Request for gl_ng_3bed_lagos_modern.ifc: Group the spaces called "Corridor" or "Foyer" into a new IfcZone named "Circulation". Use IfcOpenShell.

First a look at what the model holds.

```python
import ifcopenshell

model = ifcopenshell.open("gl_ng_3bed_lagos_modern.ifc")
print(model.schema)
seen = {}
for space in model.by_type("IfcSpace"):
    seen[space.LongName] = seen.get(space.LongName, 0) + 1
for name, count in sorted(seen.items(), key=str):
    print(count, "x", name)
print("zones:", [z.Name for z in model.by_type("IfcZone")][:20])
```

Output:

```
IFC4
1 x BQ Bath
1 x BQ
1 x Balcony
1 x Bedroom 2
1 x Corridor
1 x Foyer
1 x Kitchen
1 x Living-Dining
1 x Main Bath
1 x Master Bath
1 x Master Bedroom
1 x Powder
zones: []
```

```python
import ifcopenshell
import ifcopenshell.api.group
import ifcopenshell.api.root

model = ifcopenshell.open("gl_ng_3bed_lagos_modern.ifc")

names = {"Corridor", "Foyer"}
spaces = [s for s in model.by_type("IfcSpace") if s.LongName in names]

zone = ifcopenshell.api.root.create_entity(model, ifc_class="IfcZone", name="Circulation")
ifcopenshell.api.group.assign_group(model, products=spaces, group=zone)
print(len(spaces), "spaces in", zone.Name)

model.write("gl_ng_3bed_lagos_modern_edited.ifc")
```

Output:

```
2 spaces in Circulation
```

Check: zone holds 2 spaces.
